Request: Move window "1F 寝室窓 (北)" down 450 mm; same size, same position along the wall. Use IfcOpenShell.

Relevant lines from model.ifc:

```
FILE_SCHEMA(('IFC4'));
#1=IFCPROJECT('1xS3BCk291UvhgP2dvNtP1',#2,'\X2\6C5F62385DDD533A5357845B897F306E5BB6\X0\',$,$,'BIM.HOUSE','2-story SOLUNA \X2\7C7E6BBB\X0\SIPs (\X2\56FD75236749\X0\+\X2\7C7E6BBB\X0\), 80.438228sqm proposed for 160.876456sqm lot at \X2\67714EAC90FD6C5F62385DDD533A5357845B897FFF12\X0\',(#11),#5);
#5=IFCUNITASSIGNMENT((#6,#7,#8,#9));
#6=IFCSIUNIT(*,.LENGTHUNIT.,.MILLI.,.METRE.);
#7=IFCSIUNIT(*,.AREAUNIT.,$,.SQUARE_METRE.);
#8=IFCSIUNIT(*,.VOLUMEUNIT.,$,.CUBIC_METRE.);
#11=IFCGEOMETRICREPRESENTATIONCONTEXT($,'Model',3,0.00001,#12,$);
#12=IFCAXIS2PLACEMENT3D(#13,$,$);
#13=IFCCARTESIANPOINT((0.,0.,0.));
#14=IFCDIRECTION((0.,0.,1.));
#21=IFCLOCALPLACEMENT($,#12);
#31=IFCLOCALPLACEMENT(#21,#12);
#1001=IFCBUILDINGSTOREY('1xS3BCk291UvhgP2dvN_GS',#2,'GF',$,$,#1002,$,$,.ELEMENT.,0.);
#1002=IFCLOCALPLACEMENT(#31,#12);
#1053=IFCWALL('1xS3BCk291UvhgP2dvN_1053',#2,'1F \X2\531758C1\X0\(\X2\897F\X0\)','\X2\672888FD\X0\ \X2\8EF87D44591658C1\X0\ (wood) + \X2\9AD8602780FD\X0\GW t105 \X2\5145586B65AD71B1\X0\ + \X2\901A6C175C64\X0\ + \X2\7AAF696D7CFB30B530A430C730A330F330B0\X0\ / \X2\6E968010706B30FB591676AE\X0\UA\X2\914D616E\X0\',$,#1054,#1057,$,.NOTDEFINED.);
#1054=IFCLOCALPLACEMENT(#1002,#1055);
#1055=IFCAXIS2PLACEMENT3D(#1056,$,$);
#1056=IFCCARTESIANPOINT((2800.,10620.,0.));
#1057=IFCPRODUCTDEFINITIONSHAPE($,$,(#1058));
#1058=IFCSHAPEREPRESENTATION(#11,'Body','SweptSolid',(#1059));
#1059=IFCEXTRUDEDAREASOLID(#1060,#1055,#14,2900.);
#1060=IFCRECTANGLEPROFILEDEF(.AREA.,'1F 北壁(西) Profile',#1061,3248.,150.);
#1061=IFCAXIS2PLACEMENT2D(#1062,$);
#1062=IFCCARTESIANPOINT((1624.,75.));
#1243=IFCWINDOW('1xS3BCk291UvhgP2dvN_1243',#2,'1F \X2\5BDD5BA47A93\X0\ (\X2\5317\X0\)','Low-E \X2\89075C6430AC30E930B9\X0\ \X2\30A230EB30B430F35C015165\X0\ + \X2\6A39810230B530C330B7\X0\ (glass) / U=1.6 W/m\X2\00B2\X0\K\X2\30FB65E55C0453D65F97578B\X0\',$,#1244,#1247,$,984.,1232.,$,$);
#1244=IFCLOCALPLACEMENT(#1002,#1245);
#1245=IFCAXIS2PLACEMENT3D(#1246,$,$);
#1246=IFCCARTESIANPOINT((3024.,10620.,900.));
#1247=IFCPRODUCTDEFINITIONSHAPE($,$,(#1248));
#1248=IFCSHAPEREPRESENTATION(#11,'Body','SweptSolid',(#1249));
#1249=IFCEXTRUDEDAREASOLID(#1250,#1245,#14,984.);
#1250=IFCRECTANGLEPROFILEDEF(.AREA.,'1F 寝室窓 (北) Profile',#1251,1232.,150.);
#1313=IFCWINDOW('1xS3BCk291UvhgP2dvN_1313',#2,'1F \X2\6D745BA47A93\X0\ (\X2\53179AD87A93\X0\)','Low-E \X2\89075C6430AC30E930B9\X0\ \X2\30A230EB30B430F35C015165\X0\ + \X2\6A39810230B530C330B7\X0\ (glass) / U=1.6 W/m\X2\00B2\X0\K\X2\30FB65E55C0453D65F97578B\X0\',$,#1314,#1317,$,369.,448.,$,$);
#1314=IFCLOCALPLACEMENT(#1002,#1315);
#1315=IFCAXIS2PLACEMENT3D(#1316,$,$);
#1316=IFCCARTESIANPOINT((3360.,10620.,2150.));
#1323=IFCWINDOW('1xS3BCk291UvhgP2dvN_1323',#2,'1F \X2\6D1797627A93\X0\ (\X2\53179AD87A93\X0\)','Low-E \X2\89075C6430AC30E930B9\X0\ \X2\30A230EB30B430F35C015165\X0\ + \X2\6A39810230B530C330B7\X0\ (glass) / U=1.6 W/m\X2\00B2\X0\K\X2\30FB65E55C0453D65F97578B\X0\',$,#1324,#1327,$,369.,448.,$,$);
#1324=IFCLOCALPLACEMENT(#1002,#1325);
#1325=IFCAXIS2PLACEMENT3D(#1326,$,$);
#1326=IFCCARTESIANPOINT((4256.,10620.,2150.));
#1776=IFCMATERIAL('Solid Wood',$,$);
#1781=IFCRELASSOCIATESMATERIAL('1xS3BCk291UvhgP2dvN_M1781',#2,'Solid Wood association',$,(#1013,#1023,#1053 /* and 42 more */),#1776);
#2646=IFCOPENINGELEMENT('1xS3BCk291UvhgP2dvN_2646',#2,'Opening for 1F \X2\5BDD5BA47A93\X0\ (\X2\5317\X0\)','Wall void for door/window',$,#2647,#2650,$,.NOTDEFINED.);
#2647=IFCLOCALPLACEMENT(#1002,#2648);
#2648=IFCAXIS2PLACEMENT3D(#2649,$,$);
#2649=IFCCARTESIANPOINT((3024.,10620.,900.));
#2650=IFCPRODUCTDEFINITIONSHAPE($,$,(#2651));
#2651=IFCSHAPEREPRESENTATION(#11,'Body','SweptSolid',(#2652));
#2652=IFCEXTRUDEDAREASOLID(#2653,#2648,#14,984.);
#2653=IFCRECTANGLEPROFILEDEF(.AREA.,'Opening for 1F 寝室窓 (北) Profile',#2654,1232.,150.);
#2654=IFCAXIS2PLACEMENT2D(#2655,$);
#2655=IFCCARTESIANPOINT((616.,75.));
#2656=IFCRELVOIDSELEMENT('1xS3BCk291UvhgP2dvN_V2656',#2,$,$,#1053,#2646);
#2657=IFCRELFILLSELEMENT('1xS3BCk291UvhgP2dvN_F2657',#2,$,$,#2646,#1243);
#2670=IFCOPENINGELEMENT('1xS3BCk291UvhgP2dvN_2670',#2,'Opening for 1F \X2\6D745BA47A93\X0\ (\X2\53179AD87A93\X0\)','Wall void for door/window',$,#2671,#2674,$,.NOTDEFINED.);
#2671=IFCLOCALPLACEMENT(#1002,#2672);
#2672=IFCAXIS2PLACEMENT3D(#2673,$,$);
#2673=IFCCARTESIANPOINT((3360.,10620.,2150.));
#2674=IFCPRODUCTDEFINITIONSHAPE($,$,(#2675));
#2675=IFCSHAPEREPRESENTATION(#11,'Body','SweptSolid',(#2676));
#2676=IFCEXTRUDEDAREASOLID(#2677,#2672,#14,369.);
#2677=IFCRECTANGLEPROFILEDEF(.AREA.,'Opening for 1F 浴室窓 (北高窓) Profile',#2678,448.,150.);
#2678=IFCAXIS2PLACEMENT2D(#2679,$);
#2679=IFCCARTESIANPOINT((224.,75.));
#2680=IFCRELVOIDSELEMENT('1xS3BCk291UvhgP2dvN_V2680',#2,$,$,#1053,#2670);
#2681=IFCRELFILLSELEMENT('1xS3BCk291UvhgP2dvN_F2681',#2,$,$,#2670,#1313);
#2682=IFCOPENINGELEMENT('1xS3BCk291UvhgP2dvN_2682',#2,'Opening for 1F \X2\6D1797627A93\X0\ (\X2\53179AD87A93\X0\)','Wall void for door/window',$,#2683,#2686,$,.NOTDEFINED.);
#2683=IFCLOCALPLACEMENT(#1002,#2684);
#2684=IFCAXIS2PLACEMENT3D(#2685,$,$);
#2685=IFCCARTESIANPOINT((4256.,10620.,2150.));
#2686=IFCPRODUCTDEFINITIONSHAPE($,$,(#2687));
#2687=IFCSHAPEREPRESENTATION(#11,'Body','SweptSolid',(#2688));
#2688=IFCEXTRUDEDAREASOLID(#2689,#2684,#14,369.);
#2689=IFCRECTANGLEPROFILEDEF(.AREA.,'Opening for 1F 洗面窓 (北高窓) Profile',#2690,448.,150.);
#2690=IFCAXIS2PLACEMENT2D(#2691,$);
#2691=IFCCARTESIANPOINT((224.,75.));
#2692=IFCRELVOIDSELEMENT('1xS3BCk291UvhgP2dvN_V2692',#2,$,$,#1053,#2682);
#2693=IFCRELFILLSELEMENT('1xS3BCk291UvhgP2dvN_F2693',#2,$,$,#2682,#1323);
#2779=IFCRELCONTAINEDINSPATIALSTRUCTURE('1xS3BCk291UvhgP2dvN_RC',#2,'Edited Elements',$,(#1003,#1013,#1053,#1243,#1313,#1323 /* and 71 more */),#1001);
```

```python
import numpy as np
import ifcopenshell
import ifcopenshell.api.geometry
import ifcopenshell.util.placement
import ifcopenshell.util.unit

model = ifcopenshell.open("model.ifc")
unit_scale = ifcopenshell.util.unit.calculate_unit_scale(model)

window = model.by_guid("1xS3BCk291UvhgP2dvN_1243")
opening = window.FillsVoids[0].RelatingOpeningElement
dz = -450.0

shift = np.array([0.0, 0.0, dz])
# The window is not placed relative to its opening, so move both.
for product in (opening, window):
    matrix = ifcopenshell.util.placement.get_local_placement(product.ObjectPlacement)
    matrix[:3, 3] += shift
    ifcopenshell.api.geometry.edit_object_placement(model, product=product, matrix=matrix, is_si=False)

print(f"moved by {dz * unit_scale:+.3f} m")

model.write("model_edited.ifc")
```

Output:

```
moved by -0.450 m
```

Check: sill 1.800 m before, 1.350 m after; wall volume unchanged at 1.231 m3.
